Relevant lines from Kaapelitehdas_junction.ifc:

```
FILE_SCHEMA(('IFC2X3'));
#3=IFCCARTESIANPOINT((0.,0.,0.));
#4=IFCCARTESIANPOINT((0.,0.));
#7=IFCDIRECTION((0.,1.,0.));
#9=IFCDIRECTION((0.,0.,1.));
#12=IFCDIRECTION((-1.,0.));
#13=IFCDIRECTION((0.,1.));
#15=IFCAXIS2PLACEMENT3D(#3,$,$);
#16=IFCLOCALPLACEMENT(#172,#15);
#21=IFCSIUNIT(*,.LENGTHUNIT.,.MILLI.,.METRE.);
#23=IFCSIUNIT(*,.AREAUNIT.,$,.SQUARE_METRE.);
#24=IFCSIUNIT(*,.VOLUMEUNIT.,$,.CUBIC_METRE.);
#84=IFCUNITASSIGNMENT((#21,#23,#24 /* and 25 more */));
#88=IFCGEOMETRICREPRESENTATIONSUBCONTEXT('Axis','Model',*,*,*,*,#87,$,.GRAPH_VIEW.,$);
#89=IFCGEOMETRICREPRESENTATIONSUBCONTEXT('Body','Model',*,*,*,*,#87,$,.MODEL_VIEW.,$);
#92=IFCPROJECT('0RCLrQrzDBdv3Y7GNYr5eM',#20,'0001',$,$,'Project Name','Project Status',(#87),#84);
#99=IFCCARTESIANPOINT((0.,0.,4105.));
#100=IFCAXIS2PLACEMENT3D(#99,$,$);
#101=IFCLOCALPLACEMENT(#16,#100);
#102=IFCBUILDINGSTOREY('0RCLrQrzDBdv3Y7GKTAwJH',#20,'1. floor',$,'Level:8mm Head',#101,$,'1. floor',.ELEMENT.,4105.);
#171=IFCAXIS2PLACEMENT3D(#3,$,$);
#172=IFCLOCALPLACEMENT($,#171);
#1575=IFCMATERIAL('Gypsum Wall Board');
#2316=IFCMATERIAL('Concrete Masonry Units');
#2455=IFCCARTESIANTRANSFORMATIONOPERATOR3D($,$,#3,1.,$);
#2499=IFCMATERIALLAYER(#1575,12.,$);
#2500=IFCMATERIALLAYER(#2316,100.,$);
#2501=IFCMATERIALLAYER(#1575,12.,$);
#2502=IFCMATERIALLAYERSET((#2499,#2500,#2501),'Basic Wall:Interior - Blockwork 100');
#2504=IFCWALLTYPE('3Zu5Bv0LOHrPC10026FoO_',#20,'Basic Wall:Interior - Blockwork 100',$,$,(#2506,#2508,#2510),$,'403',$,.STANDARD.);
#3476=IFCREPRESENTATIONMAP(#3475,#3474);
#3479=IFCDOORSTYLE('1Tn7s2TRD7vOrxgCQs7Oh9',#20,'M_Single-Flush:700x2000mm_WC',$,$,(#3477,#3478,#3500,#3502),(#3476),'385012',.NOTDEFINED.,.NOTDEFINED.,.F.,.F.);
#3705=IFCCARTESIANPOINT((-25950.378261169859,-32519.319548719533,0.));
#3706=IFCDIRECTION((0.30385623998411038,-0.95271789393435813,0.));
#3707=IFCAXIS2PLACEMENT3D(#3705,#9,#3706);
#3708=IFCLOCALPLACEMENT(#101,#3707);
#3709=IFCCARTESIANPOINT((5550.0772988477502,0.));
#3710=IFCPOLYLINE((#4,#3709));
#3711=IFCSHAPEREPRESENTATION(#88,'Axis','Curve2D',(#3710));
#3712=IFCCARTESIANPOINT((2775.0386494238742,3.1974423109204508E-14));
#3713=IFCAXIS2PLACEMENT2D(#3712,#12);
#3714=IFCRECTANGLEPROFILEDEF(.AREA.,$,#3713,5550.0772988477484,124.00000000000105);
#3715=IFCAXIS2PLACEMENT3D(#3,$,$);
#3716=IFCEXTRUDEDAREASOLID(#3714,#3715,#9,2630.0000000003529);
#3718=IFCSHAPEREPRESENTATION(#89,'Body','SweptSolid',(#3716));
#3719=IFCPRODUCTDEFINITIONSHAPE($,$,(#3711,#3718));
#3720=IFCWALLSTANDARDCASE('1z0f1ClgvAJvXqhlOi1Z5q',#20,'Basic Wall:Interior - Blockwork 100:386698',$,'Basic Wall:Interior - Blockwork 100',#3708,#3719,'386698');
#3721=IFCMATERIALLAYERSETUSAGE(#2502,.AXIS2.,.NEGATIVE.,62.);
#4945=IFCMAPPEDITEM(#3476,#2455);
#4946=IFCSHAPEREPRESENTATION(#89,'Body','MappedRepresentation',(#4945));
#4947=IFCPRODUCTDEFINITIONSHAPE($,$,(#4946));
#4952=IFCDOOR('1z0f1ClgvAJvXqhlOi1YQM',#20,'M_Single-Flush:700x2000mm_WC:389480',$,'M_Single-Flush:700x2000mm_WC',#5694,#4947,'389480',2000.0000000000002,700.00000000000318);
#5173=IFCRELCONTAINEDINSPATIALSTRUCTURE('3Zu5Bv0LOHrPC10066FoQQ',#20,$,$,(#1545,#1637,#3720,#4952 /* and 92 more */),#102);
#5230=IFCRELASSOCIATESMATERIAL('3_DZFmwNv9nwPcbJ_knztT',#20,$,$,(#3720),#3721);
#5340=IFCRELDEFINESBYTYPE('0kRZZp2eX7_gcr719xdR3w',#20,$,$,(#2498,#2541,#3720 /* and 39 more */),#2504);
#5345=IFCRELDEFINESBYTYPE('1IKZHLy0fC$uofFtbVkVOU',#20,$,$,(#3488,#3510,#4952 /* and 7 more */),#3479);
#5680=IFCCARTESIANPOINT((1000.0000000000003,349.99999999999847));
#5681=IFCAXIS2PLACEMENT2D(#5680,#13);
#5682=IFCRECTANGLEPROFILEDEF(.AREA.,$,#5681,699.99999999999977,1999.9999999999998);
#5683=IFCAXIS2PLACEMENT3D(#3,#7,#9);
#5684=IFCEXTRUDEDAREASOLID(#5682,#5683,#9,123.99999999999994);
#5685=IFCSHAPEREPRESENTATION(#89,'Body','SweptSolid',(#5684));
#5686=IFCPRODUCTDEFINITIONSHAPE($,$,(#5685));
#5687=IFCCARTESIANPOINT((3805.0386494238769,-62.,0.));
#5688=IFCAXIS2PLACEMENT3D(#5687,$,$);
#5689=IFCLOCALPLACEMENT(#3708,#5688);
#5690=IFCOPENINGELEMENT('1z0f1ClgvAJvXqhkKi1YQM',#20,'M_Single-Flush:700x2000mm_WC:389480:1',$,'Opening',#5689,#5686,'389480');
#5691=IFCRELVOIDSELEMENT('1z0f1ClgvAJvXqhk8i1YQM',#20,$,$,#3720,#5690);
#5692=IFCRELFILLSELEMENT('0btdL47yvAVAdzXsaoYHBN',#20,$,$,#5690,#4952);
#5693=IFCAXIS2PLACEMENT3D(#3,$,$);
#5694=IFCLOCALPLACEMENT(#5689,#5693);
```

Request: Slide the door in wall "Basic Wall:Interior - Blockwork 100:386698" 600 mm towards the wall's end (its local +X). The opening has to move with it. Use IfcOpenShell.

```python
import ifcopenshell
import ifcopenshell.api.geometry
import ifcopenshell.util.placement
import ifcopenshell.util.unit

model = ifcopenshell.open("Kaapelitehdas_junction.ifc")
unit_scale = ifcopenshell.util.unit.calculate_unit_scale(model)

door = model.by_id(4952)
opening = door.FillsVoids[0].RelatingOpeningElement
wall = opening.VoidsElements[0].RelatingBuildingElement

wall_matrix = ifcopenshell.util.placement.get_local_placement(wall.ObjectPlacement)
shift = wall_matrix[:3, 0] * 0.6 / unit_scale
before = ifcopenshell.util.placement.get_local_placement(door.ObjectPlacement)[:3, 3].copy()

# The door is placed relative to its opening, so it follows when the opening moves.
matrix = ifcopenshell.util.placement.get_local_placement(opening.ObjectPlacement)
matrix[:3, 3] += shift
ifcopenshell.api.geometry.edit_object_placement(
    model, product=opening, matrix=matrix, is_si=False, should_transform_children=True
)

after = ifcopenshell.util.placement.get_local_placement(door.ObjectPlacement)[:3, 3]
print("door moved by", (after - before).round(3) + 0.0)

model.write("Kaapelitehdas_junction_v2.ifc")
```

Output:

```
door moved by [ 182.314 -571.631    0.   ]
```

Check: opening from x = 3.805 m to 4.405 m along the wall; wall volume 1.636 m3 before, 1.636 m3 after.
